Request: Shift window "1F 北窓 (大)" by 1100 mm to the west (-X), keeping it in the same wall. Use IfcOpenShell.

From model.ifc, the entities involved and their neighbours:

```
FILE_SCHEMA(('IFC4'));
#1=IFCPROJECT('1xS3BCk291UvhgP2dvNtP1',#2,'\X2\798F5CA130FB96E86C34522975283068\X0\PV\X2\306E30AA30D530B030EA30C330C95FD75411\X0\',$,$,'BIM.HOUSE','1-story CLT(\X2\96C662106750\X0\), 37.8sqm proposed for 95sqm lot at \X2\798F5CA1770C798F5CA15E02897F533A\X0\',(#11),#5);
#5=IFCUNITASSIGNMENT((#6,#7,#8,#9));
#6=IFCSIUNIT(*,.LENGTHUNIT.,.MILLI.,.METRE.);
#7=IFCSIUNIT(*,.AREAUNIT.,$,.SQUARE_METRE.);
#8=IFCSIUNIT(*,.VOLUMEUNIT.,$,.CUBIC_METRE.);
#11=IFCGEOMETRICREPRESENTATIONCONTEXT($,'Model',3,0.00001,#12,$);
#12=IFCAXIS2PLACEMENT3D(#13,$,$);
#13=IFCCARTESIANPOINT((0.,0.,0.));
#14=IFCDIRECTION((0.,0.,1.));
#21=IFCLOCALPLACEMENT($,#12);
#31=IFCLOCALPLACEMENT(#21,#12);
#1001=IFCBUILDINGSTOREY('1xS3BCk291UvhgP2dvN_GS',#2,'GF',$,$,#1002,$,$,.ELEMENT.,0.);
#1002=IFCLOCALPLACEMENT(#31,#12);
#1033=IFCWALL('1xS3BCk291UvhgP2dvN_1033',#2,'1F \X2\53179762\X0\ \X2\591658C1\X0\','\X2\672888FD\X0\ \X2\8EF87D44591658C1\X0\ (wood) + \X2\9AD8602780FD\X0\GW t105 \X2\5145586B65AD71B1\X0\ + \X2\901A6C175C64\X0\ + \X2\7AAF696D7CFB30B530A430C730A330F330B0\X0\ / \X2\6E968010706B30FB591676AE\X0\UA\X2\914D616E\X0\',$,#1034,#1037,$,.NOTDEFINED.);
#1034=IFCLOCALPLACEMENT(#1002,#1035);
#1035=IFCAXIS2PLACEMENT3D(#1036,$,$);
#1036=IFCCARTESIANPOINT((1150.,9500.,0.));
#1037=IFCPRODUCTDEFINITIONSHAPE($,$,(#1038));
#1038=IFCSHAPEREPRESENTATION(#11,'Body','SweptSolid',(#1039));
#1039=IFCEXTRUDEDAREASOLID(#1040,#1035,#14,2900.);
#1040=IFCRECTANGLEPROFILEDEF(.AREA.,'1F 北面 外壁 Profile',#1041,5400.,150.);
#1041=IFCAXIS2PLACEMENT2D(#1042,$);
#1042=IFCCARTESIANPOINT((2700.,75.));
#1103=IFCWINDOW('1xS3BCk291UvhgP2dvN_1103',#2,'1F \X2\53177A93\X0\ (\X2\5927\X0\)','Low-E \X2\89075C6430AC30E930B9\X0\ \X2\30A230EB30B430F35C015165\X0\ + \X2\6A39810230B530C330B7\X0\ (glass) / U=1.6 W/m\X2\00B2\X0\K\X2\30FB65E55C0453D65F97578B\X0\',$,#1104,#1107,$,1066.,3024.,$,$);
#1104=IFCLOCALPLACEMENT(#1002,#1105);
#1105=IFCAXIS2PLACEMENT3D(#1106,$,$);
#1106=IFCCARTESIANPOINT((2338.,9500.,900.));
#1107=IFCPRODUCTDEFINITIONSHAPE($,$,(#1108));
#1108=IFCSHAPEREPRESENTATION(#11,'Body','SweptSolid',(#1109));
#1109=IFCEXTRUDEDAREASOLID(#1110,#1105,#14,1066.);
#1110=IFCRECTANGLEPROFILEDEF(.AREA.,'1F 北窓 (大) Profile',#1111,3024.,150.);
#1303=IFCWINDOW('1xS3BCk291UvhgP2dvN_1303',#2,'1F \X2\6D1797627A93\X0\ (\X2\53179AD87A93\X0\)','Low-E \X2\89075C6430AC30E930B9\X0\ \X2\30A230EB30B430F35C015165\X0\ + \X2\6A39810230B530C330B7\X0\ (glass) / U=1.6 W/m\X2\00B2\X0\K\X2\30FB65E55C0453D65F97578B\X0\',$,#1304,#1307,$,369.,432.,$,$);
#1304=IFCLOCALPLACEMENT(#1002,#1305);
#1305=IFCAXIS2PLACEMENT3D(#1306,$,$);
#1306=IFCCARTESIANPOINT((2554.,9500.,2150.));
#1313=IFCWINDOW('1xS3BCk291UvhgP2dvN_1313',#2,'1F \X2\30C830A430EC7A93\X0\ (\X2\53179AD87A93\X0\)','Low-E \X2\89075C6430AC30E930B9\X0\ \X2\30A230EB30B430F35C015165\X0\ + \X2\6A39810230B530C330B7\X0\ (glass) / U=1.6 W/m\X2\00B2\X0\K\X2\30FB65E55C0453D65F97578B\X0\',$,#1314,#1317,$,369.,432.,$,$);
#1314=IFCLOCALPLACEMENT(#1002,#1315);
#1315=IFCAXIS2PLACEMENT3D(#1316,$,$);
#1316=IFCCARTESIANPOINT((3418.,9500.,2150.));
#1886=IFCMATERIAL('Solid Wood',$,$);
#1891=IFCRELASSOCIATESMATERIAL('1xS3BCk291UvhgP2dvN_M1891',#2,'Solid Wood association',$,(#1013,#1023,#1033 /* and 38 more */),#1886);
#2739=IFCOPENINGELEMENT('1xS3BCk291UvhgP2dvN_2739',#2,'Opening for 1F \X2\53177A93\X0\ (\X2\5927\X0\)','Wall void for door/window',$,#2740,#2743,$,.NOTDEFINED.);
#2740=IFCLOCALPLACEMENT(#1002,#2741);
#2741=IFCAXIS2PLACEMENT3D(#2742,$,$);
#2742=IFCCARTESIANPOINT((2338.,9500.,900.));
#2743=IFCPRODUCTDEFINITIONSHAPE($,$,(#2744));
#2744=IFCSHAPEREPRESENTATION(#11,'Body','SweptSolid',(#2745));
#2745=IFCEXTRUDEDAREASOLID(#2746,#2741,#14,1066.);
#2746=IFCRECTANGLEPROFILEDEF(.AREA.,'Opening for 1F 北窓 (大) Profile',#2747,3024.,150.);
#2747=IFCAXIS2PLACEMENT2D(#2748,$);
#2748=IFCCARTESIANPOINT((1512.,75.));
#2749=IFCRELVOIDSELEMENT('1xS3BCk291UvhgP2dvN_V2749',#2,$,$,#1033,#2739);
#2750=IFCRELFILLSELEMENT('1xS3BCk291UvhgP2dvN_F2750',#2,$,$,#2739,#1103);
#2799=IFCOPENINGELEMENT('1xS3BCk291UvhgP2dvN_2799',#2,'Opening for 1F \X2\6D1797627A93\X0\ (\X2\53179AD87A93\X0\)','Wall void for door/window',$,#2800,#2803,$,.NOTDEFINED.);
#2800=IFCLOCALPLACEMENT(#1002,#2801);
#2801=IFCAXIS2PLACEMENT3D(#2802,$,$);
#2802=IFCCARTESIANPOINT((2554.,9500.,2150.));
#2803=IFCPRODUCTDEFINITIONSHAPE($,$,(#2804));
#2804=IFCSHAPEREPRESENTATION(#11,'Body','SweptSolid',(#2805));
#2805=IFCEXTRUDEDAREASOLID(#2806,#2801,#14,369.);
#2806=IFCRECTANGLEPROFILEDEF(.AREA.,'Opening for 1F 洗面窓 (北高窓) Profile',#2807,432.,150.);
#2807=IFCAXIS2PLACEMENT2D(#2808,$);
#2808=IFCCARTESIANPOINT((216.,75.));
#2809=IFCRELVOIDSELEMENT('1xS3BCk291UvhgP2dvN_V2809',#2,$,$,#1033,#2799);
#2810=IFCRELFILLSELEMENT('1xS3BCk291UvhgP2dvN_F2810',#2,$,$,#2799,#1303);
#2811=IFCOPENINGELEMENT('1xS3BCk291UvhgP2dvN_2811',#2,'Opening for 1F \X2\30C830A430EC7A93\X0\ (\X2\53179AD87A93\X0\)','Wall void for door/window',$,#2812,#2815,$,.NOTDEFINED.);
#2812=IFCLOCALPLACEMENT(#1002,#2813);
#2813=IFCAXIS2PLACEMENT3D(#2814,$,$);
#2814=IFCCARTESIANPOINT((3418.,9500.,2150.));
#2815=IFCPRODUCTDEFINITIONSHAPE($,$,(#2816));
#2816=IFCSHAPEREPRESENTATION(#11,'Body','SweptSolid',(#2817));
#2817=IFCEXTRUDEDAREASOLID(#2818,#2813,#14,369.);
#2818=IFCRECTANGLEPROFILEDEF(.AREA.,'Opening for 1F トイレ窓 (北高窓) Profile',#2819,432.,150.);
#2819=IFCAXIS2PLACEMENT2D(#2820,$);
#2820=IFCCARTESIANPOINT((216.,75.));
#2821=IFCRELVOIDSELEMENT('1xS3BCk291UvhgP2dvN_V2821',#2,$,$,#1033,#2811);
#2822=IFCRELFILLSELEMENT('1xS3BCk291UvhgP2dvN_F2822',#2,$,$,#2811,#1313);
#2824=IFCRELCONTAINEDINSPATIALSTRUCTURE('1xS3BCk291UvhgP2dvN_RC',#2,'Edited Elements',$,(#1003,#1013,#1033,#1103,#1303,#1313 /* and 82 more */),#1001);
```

```python
import ifcopenshell
import ifcopenshell.api.geometry
import ifcopenshell.util.placement

model = ifcopenshell.open("model.ifc")

window = model.by_guid("1xS3BCk291UvhgP2dvN_1103")
opening = window.FillsVoids[0].RelatingOpeningElement
wall = opening.VoidsElements[0].RelatingBuildingElement

wall_matrix = ifcopenshell.util.placement.get_local_placement(wall.ObjectPlacement)
shift = wall_matrix[:3, 0] * -1100.0
before = ifcopenshell.util.placement.get_local_placement(window.ObjectPlacement)[:3, 3].copy()

# The window is not placed relative to its opening, so move both.
for product in (opening, window):
    matrix = ifcopenshell.util.placement.get_local_placement(product.ObjectPlacement)
    matrix[:3, 3] += shift
    ifcopenshell.api.geometry.edit_object_placement(model, product=product, matrix=matrix, is_si=False)

after = ifcopenshell.util.placement.get_local_placement(window.ObjectPlacement)[:3, 3]
print("window moved by", (after - before).round(3) + 0.0)

model.write("model_updated.ifc")
```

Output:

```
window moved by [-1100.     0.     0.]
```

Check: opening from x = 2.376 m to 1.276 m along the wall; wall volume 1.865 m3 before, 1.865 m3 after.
